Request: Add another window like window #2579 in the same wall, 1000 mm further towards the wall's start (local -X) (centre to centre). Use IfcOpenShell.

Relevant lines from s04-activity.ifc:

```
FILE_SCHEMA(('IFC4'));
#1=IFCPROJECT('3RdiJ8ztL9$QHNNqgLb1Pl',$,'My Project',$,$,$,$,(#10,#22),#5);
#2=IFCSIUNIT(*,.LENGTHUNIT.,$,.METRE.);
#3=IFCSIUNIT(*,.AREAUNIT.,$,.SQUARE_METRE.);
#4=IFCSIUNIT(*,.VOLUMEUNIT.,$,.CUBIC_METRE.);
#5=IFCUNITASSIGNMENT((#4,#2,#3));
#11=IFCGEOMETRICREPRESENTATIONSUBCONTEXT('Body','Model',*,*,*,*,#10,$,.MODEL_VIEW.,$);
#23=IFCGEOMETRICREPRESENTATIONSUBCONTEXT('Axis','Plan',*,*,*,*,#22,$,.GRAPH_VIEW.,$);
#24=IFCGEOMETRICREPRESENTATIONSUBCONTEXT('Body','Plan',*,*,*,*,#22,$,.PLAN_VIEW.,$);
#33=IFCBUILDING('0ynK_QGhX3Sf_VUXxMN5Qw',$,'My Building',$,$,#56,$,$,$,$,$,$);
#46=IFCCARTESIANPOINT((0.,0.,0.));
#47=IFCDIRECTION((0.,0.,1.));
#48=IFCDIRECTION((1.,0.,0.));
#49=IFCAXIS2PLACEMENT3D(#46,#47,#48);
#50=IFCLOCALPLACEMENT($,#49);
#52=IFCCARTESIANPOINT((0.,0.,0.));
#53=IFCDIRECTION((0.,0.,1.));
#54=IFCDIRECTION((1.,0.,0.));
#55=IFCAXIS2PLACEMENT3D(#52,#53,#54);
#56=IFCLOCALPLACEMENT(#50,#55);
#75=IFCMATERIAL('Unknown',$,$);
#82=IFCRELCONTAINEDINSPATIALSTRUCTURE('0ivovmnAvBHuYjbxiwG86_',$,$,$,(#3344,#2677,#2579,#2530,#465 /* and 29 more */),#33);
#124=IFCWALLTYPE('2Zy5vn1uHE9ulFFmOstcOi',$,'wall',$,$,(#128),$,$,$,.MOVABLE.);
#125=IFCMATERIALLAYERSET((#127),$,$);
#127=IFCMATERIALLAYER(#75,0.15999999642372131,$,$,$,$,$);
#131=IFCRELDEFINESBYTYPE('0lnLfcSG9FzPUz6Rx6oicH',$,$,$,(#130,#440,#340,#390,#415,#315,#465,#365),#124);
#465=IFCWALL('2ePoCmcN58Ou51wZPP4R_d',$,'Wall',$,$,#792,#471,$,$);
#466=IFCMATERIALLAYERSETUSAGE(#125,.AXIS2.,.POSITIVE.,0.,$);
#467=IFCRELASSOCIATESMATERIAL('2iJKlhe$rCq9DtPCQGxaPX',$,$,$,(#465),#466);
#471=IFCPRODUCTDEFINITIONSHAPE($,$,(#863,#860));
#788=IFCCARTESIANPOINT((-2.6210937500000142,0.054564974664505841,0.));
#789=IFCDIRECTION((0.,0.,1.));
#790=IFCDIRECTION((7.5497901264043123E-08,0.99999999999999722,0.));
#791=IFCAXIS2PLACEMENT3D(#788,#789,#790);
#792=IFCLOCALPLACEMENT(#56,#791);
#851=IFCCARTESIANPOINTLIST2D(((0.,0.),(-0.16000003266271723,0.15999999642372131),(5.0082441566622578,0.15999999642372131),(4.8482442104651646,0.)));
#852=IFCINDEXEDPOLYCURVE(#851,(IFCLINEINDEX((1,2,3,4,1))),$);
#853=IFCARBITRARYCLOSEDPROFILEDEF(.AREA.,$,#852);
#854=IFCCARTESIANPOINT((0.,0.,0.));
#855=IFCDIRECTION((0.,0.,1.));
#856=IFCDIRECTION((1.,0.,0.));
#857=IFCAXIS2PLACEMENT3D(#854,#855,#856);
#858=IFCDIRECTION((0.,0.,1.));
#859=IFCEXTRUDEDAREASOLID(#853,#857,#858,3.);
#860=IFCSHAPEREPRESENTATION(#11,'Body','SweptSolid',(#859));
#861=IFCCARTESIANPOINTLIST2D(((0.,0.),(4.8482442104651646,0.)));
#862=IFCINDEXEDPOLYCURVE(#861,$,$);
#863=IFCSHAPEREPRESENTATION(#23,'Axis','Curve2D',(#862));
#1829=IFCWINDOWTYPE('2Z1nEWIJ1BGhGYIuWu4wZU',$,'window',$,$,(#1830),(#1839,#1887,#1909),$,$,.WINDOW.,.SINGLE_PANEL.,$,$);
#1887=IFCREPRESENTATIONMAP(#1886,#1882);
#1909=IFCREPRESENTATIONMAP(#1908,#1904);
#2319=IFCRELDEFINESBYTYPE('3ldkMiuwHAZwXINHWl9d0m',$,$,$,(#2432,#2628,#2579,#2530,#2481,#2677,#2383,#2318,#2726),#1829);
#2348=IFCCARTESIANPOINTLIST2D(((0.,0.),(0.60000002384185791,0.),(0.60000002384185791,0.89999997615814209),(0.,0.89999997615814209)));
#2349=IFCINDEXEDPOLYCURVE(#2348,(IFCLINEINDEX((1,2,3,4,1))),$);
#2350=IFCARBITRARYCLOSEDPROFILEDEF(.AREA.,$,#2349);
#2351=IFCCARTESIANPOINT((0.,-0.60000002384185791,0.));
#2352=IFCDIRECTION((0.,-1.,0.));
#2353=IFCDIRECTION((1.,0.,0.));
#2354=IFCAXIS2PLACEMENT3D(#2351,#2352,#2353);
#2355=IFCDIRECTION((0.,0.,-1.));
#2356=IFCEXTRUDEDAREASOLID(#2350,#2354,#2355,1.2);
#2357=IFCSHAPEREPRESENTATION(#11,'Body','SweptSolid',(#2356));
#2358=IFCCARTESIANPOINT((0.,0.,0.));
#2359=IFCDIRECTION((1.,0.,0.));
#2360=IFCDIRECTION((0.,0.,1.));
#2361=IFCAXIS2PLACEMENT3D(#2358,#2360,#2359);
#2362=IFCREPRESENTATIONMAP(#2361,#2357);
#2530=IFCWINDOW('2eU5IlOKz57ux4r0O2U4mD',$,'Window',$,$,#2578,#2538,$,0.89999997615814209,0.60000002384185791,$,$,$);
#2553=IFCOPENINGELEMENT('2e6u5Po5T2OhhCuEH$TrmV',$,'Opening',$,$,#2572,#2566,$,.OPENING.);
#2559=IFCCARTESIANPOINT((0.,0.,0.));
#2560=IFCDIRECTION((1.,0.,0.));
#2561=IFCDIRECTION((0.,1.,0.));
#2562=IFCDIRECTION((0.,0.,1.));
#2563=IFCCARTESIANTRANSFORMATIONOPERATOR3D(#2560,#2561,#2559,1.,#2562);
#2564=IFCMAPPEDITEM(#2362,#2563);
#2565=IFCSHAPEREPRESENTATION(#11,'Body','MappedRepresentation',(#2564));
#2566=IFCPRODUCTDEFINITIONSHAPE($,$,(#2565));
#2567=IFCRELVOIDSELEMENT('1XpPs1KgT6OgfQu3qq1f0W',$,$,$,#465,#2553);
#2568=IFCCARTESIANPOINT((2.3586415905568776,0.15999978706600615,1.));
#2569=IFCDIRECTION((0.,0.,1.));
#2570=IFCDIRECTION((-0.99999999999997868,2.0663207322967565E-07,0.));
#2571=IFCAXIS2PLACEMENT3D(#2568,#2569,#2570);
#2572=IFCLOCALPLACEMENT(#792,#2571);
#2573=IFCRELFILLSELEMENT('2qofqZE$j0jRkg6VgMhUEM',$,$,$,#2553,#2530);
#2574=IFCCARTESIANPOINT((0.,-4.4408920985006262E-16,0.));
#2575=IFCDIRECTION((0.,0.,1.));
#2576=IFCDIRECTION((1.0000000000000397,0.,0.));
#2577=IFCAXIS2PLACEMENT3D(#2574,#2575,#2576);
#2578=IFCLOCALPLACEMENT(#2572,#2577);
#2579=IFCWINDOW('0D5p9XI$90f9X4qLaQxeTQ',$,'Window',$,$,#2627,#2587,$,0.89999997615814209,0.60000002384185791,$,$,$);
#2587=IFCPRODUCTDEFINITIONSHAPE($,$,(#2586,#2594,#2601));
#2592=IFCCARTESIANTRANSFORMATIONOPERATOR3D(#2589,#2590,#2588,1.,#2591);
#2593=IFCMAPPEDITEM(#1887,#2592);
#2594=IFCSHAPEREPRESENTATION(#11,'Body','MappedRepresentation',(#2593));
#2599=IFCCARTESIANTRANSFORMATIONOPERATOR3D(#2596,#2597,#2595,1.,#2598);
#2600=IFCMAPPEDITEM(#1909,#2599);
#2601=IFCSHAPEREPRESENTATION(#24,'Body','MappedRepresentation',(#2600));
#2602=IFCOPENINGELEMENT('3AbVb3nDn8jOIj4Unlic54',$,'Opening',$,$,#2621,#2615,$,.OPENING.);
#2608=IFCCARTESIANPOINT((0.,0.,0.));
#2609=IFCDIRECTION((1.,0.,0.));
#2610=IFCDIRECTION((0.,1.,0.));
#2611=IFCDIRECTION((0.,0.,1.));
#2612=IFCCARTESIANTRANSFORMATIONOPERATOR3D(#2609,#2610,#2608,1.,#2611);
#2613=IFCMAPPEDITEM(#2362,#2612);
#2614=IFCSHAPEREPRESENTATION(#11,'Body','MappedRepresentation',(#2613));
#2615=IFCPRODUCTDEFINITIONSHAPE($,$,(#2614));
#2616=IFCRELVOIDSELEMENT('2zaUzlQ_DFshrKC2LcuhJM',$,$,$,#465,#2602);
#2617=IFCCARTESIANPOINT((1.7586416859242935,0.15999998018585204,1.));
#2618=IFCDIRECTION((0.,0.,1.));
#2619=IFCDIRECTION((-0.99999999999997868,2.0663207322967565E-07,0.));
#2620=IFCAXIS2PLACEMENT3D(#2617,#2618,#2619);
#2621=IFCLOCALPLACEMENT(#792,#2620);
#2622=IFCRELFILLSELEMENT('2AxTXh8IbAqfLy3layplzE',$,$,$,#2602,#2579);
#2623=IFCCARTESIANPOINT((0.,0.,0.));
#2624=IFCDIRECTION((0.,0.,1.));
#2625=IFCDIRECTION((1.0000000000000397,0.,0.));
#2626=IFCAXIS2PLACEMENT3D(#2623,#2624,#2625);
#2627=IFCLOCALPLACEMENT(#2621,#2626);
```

```python
import ifcopenshell
import ifcopenshell.api.feature
import ifcopenshell.api.geometry
import ifcopenshell.api.root
import ifcopenshell.geom
import ifcopenshell.util.element
import ifcopenshell.util.placement
import ifcopenshell.util.shape
import ifcopenshell.util.unit

model = ifcopenshell.open("s04-activity.ifc")
unit_scale = ifcopenshell.util.unit.calculate_unit_scale(model)
settings = ifcopenshell.geom.settings()


def volume(element):
    """Net volume in cubic metres, openings subtracted."""
    shape = ifcopenshell.geom.create_shape(settings, element)
    return ifcopenshell.util.shape.get_volume(shape.geometry)


window = model.by_guid("0D5p9XI$90f9X4qLaQxeTQ")
opening = window.FillsVoids[0].RelatingOpeningElement
wall = opening.VoidsElements[0].RelatingBuildingElement
before = volume(wall)
shift = ifcopenshell.util.placement.get_local_placement(wall.ObjectPlacement)[:3, 0] * -1 / unit_scale

# copy_class copies the void relationship, type, container and properties, but no geometry.
new_opening = ifcopenshell.api.root.copy_class(model, product=opening)
new_opening.Representation = ifcopenshell.util.element.copy_deep(
    model, opening.Representation, exclude=["IfcGeometricRepresentationContext", "IfcRepresentationMap"]
)
new_window = ifcopenshell.api.root.copy_class(model, product=window)
new_window.Representation = ifcopenshell.util.element.copy_deep(
    model, window.Representation, exclude=["IfcGeometricRepresentationContext", "IfcRepresentationMap"]
)
ifcopenshell.api.feature.add_filling(model, opening=new_opening, element=new_window)

for old, new in ((opening, new_opening), (window, new_window)):
    matrix = ifcopenshell.util.placement.get_local_placement(old.ObjectPlacement)
    matrix[:3, 3] += shift
    ifcopenshell.api.geometry.edit_object_placement(model, product=new, matrix=matrix, is_si=False)

after = volume(wall)

print(f"wall volume {before:.3f} -> {after:.3f} m3")

model.write("s04-activity_rev.ifc")
```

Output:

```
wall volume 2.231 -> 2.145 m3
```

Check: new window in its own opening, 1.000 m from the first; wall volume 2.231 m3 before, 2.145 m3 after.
